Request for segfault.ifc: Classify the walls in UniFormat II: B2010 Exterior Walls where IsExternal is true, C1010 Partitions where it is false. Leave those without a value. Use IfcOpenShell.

First a look at what the model holds.

```python
import ifcopenshell
import ifcopenshell.util.element

model = ifcopenshell.open("segfault.ifc")
print(model.schema)
print("classifications:", [c.Name for c in model.by_type("IfcClassification")])
values = [ifcopenshell.util.element.get_pset(e, "Pset_WallCommon", "IsExternal") for e in model.by_type("IfcWall")]
for value in (True, False, None):
    print("IsExternal", value, values.count(value))
```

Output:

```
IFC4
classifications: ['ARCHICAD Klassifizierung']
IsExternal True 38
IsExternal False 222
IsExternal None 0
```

```python
import ifcopenshell
import ifcopenshell.api.classification
import ifcopenshell.util.element

model = ifcopenshell.open("segfault.ifc")

system = ifcopenshell.api.classification.add_classification(model, classification="UniFormat II")

walls = model.by_type("IfcWall")
external = {e: ifcopenshell.util.element.get_pset(e, "Pset_WallCommon", "IsExternal") for e in walls}
for flag, code, name in ((True, "B2010", "Exterior Walls"), (False, "C1010", "Partitions")):
    products = [e for e in walls if external[e] is flag]
    ifcopenshell.api.classification.add_reference(
        model, products=products, classification=system, identification=code, name=name
    )
    print(code, len(products))

model.write("segfault_updated.ifc")
```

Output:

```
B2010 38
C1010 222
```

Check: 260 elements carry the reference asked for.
